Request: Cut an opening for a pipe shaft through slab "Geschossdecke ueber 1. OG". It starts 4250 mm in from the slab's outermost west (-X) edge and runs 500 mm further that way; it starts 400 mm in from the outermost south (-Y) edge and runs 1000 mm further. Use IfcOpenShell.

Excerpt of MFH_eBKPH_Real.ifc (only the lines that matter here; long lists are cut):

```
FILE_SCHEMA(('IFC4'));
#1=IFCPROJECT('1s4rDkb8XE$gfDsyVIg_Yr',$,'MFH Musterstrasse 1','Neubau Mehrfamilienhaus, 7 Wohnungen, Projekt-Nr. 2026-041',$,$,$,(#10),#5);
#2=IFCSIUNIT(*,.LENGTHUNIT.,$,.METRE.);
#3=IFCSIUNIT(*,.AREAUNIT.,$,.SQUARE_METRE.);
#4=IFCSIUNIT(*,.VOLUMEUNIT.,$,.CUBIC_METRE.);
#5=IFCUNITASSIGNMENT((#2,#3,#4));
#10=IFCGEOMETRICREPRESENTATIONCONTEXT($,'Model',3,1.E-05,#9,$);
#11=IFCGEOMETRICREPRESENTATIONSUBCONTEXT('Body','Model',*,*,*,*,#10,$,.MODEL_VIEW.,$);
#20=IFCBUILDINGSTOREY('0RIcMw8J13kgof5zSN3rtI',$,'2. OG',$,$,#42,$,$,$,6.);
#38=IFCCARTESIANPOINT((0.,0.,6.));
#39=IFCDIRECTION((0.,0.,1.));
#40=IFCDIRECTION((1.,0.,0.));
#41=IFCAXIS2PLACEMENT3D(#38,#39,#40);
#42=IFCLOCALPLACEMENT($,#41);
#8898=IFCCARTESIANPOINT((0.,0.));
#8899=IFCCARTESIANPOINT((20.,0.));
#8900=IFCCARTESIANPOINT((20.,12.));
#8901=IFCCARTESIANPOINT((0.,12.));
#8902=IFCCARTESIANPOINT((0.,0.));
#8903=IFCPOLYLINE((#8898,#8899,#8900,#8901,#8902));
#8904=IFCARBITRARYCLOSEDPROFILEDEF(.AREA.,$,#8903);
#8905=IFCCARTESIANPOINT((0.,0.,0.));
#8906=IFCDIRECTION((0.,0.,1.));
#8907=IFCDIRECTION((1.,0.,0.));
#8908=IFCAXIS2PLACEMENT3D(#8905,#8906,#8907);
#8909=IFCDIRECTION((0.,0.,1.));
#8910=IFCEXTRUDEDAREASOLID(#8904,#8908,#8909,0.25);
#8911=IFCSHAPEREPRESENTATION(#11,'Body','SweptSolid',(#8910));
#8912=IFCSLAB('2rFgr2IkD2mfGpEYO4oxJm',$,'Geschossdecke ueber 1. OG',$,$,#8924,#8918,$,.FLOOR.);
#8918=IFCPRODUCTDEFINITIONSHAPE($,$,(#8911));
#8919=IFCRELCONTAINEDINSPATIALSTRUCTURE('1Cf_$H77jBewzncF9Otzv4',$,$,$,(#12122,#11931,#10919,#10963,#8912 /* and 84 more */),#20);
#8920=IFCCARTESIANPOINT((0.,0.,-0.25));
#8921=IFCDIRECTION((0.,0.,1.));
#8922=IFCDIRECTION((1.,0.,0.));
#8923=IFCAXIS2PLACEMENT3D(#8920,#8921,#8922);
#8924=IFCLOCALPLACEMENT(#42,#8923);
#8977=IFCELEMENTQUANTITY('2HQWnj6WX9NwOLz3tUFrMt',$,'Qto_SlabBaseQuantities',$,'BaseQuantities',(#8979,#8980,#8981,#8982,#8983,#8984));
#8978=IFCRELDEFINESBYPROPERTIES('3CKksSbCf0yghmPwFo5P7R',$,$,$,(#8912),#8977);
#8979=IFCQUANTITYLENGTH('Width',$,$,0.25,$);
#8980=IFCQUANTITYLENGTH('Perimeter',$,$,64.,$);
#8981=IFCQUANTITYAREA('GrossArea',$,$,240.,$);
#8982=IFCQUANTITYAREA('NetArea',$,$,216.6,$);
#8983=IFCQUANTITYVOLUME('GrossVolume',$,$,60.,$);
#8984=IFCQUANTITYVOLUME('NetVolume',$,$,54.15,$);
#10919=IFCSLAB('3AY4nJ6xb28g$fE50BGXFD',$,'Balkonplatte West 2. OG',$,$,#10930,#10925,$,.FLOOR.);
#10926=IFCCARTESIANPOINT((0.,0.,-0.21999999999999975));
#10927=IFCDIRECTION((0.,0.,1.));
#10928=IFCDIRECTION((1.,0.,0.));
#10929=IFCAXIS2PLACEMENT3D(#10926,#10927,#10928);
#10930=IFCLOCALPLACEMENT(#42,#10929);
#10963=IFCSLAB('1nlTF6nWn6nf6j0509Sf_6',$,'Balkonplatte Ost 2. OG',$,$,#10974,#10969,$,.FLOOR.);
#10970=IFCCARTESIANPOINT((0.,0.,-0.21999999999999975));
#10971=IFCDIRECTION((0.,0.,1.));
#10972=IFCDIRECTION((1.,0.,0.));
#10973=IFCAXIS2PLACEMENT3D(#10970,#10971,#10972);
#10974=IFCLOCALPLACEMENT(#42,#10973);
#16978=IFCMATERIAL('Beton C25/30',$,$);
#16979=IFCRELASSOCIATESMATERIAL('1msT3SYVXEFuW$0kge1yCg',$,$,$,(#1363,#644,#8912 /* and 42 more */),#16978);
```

```python
import numpy as np
import ifcopenshell
import ifcopenshell.api.feature
import ifcopenshell.api.geometry
import ifcopenshell.api.pset
import ifcopenshell.api.root
import ifcopenshell.geom
import ifcopenshell.util.element
import ifcopenshell.util.placement
import ifcopenshell.util.representation
import ifcopenshell.util.shape
import ifcopenshell.util.unit

model = ifcopenshell.open("MFH_eBKPH_Real.ifc")
unit_scale = ifcopenshell.util.unit.calculate_unit_scale(model)
area_scale = ifcopenshell.util.unit.calculate_unit_scale(model, "AREAUNIT")
volume_scale = ifcopenshell.util.unit.calculate_unit_scale(model, "VOLUMEUNIT")
settings = ifcopenshell.geom.settings()


def volume(element):
    """Net volume in cubic metres, openings subtracted."""
    shape = ifcopenshell.geom.create_shape(settings, element)
    return ifcopenshell.util.shape.get_volume(shape.geometry)


slab = model.by_guid("2rFgr2IkD2mfGpEYO4oxJm")
before = volume(slab)

# Extent in the slab's own axes, in metres. The edges named are its -X and -Y sides.
slab_shape = ifcopenshell.geom.create_shape(settings, slab)
vertices = ifcopenshell.util.shape.get_vertices(slab_shape.geometry)
x_min, y_min, bottom = vertices.min(axis=0)
top = vertices[:, 2].max()

opening = ifcopenshell.api.root.create_entity(model, ifc_class="IfcOpeningElement", name="Pipe shaft opening", predefined_type="OPENING")
context = ifcopenshell.util.representation.get_context(model, "Model", "Body", "MODEL_VIEW")
width, depth = 0.5, 1
outline = [(0.0, 0.0), (width, 0.0), (width, depth), (0.0, depth), (0.0, 0.0)]
# Overshoot both faces by 50 mm so the cut is clean.
shape = ifcopenshell.api.geometry.add_slab_representation(
    model, context=context, depth=top - bottom + 0.1, polyline=outline
)
ifcopenshell.api.geometry.assign_representation(model, product=opening, representation=shape)

matrix = ifcopenshell.util.placement.get_local_placement(slab.ObjectPlacement)
matrix[:, 3] = matrix @ np.append(np.array([x_min + 4.25, y_min + 0.4, bottom - 0.05]) / unit_scale, 1.0)
ifcopenshell.api.geometry.edit_object_placement(model, product=opening, matrix=matrix, is_si=False)
ifcopenshell.api.feature.add_feature(model, feature=opening, element=slab)

after = volume(slab)

# Update the slab's stored quantities.
qto = model.by_id(ifcopenshell.util.element.get_pset(slab, "Qto_SlabBaseQuantities", should_inherit=False)["id"])
ifcopenshell.api.pset.edit_qto(model, qto=qto, properties={
    "NetArea": after / (top - bottom) / area_scale,
    "NetVolume": after / volume_scale,
})

print(f"slab volume {before:.3f} -> {after:.3f} m3")

model.write("MFH_eBKPH_Real_rev.ifc")
```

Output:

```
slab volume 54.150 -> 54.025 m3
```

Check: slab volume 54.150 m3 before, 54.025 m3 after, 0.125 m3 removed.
